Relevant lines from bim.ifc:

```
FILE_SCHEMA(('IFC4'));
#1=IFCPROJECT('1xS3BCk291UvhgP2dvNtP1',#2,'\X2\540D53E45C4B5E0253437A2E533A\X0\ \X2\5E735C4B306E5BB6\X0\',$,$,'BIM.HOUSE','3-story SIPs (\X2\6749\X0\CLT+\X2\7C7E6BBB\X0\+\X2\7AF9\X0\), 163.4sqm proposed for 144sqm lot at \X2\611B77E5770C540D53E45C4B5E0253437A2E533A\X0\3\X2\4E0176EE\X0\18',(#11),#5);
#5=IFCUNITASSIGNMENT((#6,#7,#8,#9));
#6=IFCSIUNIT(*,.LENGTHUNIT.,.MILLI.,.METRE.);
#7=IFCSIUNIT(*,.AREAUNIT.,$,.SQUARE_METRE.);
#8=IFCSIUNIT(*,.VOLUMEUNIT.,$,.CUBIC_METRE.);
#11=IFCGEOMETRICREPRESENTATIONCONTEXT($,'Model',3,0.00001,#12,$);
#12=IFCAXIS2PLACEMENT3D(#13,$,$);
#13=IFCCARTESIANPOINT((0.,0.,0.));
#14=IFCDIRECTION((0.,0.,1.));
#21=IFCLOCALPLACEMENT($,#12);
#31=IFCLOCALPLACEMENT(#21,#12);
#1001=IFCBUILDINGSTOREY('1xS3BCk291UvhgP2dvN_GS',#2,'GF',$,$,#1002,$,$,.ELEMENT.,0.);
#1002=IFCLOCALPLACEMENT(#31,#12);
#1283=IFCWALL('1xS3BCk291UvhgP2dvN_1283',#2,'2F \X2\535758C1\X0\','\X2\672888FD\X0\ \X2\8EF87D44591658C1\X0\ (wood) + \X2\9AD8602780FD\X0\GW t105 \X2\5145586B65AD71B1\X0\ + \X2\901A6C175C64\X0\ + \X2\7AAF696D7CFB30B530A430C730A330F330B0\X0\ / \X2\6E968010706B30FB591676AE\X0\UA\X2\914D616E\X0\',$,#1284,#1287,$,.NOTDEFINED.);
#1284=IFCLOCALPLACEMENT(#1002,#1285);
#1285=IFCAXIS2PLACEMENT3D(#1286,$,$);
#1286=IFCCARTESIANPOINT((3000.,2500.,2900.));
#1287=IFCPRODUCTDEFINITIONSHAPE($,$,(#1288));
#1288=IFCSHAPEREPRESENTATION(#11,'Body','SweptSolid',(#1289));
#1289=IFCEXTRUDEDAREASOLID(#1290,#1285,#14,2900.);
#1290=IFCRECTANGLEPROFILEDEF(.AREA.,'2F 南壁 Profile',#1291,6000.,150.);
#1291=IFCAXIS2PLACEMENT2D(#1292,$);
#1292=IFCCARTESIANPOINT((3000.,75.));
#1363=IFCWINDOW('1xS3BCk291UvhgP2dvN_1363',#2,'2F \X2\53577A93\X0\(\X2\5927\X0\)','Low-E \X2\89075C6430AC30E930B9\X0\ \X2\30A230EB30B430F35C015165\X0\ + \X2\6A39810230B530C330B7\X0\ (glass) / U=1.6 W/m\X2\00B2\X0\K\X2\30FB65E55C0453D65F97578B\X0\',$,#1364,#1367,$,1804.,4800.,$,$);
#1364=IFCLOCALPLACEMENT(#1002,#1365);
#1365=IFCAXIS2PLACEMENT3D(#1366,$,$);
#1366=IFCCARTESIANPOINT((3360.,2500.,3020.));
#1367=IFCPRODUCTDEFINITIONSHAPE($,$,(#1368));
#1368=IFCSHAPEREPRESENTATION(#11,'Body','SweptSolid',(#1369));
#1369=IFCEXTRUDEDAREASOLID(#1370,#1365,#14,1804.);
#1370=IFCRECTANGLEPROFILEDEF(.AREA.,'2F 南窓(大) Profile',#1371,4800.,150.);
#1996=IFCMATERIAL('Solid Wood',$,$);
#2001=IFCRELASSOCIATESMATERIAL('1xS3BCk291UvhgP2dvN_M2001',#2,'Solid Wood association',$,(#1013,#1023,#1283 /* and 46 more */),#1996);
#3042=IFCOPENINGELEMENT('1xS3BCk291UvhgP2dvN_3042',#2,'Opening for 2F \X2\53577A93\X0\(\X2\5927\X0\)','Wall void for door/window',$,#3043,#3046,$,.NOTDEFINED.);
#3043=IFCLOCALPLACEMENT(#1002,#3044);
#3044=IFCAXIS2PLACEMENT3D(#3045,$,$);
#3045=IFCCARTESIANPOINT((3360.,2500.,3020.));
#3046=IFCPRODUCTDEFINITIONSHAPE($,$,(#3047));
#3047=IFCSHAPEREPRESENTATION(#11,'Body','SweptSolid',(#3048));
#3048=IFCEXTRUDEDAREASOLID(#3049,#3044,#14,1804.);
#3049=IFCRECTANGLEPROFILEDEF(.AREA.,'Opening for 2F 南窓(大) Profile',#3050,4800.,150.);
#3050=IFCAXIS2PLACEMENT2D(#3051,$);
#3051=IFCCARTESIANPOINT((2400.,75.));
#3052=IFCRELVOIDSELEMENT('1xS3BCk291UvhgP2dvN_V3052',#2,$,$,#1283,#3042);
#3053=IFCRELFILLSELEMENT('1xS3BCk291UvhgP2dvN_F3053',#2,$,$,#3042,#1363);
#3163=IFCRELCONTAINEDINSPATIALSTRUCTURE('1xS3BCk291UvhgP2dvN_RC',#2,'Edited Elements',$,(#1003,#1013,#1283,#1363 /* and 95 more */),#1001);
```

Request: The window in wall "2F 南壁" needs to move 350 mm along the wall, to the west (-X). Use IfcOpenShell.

```python
import ifcopenshell
import ifcopenshell.api.geometry
import ifcopenshell.util.placement
import ifcopenshell.util.unit

model = ifcopenshell.open("bim.ifc")
unit_scale = ifcopenshell.util.unit.calculate_unit_scale(model)

window = model.by_guid("1xS3BCk291UvhgP2dvN_1363")
opening = window.FillsVoids[0].RelatingOpeningElement
wall = opening.VoidsElements[0].RelatingBuildingElement

wall_matrix = ifcopenshell.util.placement.get_local_placement(wall.ObjectPlacement)
shift = wall_matrix[:3, 0] * -0.35 / unit_scale
before = ifcopenshell.util.placement.get_local_placement(window.ObjectPlacement)[:3, 3].copy()

# The window is not placed relative to its opening, so move both.
for product in (opening, window):
    matrix = ifcopenshell.util.placement.get_local_placement(product.ObjectPlacement)
    matrix[:3, 3] += shift
    ifcopenshell.api.geometry.edit_object_placement(model, product=product, matrix=matrix, is_si=False)

after = ifcopenshell.util.placement.get_local_placement(window.ObjectPlacement)[:3, 3]
print("window moved by", (after - before).round(3) + 0.0)

model.write("bim_edited.ifc")
```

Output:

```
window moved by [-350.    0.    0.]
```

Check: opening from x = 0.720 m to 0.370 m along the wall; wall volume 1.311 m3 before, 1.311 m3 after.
